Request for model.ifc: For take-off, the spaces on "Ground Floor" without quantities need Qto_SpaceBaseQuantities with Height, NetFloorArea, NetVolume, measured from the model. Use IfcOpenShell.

First a look at what the model holds.

```python
import ifcopenshell
import ifcopenshell.util.element
import ifcopenshell.util.unit

model = ifcopenshell.open("model.ifc")
print(model.schema)
for unit_type in ("LENGTHUNIT", "AREAUNIT", "VOLUMEUNIT"):
    print(unit_type, ifcopenshell.util.unit.calculate_unit_scale(model, unit_type))
storey = next(s for s in model.by_type("IfcBuildingStorey") if s.Name == "Ground Floor")
spaces = [e for e in ifcopenshell.util.element.get_decomposition(storey) if e.is_a("IfcSpace")]
for e in sorted(spaces, key=lambda e: e.id()):
    print(e.id(), e.is_a(), e.Name, list(ifcopenshell.util.element.get_psets(e, qtos_only=True)), sep=" | ")
```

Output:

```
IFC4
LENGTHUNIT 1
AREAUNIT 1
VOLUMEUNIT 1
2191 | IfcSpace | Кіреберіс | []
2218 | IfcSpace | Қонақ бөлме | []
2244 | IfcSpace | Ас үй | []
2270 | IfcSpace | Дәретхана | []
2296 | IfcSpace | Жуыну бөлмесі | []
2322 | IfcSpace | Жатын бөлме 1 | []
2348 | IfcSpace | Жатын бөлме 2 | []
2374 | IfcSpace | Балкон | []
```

```python
import ifcopenshell
import ifcopenshell.api.pset
import ifcopenshell.geom
import ifcopenshell.util.element
import ifcopenshell.util.shape
import ifcopenshell.util.unit

model = ifcopenshell.open("model.ifc")
unit_scale = ifcopenshell.util.unit.calculate_unit_scale(model)
area_scale = ifcopenshell.util.unit.calculate_unit_scale(model, "AREAUNIT")
volume_scale = ifcopenshell.util.unit.calculate_unit_scale(model, "VOLUMEUNIT")
settings = ifcopenshell.geom.settings()

storey = next(s for s in model.by_type("IfcBuildingStorey") if s.Name == "Ground Floor")
spaces = [e for e in ifcopenshell.util.element.get_decomposition(storey) if e.is_a("IfcSpace")]

for e in sorted(spaces, key=lambda e: e.id()):
    if ifcopenshell.util.element.get_psets(e, qtos_only=True, should_inherit=False):
        continue
    # Geometry comes back in metres, in the element's own axes.
    shape = ifcopenshell.geom.create_shape(settings, e)
    values = {
        "Height": ifcopenshell.util.shape.get_z(shape.geometry) / unit_scale,
        "NetFloorArea": ifcopenshell.util.shape.get_footprint_area(shape.geometry) / area_scale,
        "NetVolume": ifcopenshell.util.shape.get_volume(shape.geometry) / volume_scale,
    }
    qto = ifcopenshell.api.pset.add_qto(model, product=e, name="Qto_SpaceBaseQuantities")
    ifcopenshell.api.pset.edit_qto(model, qto=qto, properties=values)
    print(e.id(), {k: round(v, 3) for k, v in values.items()})

model.write("model_updated.ifc")
```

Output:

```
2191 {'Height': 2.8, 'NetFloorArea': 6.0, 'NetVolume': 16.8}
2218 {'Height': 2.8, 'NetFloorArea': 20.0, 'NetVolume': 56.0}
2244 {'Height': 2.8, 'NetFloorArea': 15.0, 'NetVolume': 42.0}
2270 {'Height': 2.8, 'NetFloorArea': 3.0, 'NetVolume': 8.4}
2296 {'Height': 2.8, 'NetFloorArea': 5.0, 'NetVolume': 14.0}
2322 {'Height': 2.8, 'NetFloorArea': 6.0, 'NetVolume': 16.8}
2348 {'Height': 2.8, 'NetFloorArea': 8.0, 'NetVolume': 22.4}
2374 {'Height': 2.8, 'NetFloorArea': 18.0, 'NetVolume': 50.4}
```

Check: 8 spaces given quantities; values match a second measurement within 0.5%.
